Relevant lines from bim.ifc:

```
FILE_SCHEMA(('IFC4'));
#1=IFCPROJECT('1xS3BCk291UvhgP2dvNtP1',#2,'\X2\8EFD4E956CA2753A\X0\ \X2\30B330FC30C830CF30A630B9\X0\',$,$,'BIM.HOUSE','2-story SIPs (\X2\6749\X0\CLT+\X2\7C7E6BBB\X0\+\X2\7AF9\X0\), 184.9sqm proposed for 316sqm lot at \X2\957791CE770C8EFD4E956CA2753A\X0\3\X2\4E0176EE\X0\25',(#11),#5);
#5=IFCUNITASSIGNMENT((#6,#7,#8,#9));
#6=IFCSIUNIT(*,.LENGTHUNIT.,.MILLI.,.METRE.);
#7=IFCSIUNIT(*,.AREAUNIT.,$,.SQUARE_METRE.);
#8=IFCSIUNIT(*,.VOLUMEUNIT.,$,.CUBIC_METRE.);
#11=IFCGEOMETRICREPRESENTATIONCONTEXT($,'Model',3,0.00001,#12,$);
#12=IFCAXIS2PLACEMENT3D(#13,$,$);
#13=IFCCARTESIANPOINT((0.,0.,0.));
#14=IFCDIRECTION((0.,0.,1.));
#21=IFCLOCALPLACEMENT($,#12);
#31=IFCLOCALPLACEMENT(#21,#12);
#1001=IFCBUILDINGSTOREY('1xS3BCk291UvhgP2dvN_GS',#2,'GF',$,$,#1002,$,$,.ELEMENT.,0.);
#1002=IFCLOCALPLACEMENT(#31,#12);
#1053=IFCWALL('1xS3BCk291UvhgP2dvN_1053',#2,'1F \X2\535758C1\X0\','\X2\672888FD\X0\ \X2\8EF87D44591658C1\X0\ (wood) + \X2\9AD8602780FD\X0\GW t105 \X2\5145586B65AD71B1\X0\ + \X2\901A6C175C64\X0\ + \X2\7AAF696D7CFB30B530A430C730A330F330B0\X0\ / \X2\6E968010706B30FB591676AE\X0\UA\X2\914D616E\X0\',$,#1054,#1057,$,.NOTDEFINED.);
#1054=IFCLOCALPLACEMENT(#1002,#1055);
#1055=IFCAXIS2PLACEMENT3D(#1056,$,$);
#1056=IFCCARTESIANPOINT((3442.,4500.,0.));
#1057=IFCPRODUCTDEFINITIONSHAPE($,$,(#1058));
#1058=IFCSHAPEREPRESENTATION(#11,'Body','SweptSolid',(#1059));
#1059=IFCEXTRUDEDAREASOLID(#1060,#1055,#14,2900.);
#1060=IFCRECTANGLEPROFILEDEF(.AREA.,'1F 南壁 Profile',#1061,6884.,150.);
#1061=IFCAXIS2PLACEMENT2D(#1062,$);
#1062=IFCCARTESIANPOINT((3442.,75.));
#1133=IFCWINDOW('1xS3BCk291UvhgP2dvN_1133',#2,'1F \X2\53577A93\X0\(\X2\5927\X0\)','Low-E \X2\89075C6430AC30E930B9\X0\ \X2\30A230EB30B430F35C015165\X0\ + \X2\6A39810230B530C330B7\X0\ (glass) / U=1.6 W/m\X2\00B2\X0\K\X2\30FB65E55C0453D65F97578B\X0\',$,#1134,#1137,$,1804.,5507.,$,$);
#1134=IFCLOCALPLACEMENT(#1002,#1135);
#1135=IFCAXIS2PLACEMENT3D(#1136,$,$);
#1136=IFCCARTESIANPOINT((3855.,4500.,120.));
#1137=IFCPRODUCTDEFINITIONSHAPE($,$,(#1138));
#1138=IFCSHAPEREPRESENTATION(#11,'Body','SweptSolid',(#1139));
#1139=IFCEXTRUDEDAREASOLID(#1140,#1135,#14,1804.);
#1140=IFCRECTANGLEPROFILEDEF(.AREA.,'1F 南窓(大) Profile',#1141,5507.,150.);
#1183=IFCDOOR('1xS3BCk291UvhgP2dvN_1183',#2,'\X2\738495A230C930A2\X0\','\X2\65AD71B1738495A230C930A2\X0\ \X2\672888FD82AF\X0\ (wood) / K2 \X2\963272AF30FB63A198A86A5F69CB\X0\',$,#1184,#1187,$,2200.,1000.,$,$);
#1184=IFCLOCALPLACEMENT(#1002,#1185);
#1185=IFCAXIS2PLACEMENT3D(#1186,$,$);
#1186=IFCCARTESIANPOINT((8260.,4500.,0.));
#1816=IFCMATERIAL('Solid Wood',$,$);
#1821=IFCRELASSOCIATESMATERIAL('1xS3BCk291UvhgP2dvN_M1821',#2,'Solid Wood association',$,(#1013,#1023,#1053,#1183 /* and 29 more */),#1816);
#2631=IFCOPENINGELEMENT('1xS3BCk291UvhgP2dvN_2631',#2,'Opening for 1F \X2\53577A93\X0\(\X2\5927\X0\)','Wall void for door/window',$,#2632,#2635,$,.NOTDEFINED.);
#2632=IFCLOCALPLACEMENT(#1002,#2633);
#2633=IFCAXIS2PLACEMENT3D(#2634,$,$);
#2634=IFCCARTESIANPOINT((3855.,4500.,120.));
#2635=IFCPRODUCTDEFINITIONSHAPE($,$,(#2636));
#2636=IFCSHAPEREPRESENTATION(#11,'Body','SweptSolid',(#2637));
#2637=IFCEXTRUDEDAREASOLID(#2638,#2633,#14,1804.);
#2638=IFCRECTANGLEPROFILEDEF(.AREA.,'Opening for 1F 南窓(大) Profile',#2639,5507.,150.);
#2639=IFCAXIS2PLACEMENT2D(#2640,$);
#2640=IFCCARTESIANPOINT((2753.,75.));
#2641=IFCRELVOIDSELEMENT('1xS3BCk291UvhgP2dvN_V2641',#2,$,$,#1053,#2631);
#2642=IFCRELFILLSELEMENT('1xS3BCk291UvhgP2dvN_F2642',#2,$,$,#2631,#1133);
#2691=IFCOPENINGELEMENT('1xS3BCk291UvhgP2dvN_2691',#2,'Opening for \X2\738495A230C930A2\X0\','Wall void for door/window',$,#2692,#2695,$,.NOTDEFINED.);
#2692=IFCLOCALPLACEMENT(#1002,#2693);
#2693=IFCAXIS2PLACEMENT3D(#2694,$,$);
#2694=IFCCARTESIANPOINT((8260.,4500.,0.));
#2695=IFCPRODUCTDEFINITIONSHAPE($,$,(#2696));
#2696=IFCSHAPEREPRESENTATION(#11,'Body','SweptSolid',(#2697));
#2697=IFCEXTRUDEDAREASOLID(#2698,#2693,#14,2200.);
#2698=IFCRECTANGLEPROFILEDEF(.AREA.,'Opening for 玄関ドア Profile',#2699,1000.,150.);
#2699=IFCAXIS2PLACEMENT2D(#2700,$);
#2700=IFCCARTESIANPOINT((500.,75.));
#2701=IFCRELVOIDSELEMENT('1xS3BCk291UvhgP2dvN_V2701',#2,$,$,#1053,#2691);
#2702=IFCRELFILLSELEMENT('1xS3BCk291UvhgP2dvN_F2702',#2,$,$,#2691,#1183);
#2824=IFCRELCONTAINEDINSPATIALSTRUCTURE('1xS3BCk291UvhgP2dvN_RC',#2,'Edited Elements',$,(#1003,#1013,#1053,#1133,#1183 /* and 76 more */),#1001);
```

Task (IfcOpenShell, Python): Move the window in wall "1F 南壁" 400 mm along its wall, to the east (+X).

```python
import ifcopenshell
import ifcopenshell.api.geometry
import ifcopenshell.util.placement
import ifcopenshell.util.unit

model = ifcopenshell.open("bim.ifc")
unit_scale = ifcopenshell.util.unit.calculate_unit_scale(model)

window = model.by_guid("1xS3BCk291UvhgP2dvN_1133")
opening = window.FillsVoids[0].RelatingOpeningElement
wall = opening.VoidsElements[0].RelatingBuildingElement

wall_matrix = ifcopenshell.util.placement.get_local_placement(wall.ObjectPlacement)
shift = wall_matrix[:3, 0] * 0.4 / unit_scale
before = ifcopenshell.util.placement.get_local_placement(window.ObjectPlacement)[:3, 3].copy()

# The window is not placed relative to its opening, so move both.
for product in (opening, window):
    matrix = ifcopenshell.util.placement.get_local_placement(product.ObjectPlacement)
    matrix[:3, 3] += shift
    ifcopenshell.api.geometry.edit_object_placement(model, product=product, matrix=matrix, is_si=False)

after = ifcopenshell.util.placement.get_local_placement(window.ObjectPlacement)[:3, 3]
print("window moved by", (after - before).round(3) + 0.0)

model.write("bim_v2.ifc")
```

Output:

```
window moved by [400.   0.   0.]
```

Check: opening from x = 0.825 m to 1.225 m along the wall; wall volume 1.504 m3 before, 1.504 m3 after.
